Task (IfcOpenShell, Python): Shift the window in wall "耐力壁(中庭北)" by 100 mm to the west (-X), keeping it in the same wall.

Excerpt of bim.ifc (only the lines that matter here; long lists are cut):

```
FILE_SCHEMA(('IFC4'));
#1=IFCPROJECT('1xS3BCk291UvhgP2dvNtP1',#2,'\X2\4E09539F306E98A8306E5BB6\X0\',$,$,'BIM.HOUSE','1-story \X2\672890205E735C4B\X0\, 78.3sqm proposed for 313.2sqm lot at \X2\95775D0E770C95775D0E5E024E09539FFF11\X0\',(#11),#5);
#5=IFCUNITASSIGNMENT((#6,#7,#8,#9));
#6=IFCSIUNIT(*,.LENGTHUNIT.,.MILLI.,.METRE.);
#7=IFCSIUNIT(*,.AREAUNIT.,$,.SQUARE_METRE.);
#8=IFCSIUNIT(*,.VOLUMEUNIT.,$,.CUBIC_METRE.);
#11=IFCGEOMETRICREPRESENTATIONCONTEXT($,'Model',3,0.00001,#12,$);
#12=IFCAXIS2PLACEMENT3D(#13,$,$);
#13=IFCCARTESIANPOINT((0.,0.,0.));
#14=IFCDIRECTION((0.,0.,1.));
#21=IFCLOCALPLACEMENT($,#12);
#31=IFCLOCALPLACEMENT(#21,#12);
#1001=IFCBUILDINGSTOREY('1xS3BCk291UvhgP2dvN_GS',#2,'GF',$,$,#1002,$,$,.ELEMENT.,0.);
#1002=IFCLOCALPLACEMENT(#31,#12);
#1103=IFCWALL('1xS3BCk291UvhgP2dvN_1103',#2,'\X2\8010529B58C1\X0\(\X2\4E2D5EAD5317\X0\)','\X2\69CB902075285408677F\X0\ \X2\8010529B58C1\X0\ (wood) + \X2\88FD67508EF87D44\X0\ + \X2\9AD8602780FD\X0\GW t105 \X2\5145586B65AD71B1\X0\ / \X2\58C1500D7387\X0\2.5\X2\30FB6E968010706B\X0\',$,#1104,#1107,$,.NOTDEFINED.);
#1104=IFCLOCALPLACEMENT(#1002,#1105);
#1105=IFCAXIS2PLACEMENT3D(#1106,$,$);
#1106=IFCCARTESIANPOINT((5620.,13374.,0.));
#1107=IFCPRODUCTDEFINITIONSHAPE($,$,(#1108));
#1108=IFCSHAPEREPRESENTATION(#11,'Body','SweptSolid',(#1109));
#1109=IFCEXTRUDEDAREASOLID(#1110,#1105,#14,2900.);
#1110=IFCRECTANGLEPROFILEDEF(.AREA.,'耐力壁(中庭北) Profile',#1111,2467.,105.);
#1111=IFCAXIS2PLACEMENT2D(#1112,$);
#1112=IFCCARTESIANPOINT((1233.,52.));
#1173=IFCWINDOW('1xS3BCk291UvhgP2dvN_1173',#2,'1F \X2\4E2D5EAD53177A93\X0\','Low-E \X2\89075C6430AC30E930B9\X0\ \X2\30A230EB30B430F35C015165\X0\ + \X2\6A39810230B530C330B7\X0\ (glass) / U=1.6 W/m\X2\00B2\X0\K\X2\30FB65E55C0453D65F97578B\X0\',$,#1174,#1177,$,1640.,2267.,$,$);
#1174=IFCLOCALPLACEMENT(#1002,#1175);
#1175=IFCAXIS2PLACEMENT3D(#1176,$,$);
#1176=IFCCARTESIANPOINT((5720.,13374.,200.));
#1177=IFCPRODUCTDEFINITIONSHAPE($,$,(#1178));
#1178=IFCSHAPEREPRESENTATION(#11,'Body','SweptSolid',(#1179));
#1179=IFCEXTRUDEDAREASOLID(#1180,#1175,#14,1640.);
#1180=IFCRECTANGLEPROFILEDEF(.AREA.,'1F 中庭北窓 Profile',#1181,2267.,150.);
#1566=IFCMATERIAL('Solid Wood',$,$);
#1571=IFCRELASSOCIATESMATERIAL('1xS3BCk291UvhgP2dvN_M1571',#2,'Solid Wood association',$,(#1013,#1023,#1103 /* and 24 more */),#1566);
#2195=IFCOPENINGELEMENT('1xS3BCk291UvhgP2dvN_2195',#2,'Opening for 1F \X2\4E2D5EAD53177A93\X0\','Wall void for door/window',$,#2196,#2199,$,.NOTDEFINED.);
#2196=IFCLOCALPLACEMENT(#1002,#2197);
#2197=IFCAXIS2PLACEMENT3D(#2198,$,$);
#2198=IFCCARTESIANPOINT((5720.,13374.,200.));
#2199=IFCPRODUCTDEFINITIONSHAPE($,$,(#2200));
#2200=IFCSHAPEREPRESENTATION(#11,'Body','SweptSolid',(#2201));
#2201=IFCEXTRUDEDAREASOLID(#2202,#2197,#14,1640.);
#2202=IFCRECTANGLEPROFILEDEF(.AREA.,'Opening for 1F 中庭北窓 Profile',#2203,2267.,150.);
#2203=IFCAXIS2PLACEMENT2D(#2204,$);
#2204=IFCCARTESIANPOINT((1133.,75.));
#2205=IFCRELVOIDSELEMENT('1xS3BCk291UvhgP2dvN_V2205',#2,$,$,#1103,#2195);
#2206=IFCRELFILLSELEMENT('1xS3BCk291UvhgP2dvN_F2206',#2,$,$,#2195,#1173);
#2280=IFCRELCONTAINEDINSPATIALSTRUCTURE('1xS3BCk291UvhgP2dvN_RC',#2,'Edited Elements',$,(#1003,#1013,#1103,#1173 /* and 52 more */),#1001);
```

```python
import ifcopenshell
import ifcopenshell.api.geometry
import ifcopenshell.util.placement
import ifcopenshell.util.unit

model = ifcopenshell.open("bim.ifc")
unit_scale = ifcopenshell.util.unit.calculate_unit_scale(model)

window = model.by_id(1173)
opening = window.FillsVoids[0].RelatingOpeningElement
wall = opening.VoidsElements[0].RelatingBuildingElement

wall_matrix = ifcopenshell.util.placement.get_local_placement(wall.ObjectPlacement)
shift = wall_matrix[:3, 0] * -0.1 / unit_scale
before = ifcopenshell.util.placement.get_local_placement(window.ObjectPlacement)[:3, 3].copy()

# The window is not placed relative to its opening, so move both.
for product in (opening, window):
    matrix = ifcopenshell.util.placement.get_local_placement(product.ObjectPlacement)
    matrix[:3, 3] += shift
    ifcopenshell.api.geometry.edit_object_placement(model, product=product, matrix=matrix, is_si=False)

after = ifcopenshell.util.placement.get_local_placement(window.ObjectPlacement)[:3, 3]
print("window moved by", (after - before).round(3) + 0.0)

model.write("bim_rev.ifc")
```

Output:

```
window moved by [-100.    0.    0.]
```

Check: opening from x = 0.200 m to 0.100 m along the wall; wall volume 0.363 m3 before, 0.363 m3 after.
